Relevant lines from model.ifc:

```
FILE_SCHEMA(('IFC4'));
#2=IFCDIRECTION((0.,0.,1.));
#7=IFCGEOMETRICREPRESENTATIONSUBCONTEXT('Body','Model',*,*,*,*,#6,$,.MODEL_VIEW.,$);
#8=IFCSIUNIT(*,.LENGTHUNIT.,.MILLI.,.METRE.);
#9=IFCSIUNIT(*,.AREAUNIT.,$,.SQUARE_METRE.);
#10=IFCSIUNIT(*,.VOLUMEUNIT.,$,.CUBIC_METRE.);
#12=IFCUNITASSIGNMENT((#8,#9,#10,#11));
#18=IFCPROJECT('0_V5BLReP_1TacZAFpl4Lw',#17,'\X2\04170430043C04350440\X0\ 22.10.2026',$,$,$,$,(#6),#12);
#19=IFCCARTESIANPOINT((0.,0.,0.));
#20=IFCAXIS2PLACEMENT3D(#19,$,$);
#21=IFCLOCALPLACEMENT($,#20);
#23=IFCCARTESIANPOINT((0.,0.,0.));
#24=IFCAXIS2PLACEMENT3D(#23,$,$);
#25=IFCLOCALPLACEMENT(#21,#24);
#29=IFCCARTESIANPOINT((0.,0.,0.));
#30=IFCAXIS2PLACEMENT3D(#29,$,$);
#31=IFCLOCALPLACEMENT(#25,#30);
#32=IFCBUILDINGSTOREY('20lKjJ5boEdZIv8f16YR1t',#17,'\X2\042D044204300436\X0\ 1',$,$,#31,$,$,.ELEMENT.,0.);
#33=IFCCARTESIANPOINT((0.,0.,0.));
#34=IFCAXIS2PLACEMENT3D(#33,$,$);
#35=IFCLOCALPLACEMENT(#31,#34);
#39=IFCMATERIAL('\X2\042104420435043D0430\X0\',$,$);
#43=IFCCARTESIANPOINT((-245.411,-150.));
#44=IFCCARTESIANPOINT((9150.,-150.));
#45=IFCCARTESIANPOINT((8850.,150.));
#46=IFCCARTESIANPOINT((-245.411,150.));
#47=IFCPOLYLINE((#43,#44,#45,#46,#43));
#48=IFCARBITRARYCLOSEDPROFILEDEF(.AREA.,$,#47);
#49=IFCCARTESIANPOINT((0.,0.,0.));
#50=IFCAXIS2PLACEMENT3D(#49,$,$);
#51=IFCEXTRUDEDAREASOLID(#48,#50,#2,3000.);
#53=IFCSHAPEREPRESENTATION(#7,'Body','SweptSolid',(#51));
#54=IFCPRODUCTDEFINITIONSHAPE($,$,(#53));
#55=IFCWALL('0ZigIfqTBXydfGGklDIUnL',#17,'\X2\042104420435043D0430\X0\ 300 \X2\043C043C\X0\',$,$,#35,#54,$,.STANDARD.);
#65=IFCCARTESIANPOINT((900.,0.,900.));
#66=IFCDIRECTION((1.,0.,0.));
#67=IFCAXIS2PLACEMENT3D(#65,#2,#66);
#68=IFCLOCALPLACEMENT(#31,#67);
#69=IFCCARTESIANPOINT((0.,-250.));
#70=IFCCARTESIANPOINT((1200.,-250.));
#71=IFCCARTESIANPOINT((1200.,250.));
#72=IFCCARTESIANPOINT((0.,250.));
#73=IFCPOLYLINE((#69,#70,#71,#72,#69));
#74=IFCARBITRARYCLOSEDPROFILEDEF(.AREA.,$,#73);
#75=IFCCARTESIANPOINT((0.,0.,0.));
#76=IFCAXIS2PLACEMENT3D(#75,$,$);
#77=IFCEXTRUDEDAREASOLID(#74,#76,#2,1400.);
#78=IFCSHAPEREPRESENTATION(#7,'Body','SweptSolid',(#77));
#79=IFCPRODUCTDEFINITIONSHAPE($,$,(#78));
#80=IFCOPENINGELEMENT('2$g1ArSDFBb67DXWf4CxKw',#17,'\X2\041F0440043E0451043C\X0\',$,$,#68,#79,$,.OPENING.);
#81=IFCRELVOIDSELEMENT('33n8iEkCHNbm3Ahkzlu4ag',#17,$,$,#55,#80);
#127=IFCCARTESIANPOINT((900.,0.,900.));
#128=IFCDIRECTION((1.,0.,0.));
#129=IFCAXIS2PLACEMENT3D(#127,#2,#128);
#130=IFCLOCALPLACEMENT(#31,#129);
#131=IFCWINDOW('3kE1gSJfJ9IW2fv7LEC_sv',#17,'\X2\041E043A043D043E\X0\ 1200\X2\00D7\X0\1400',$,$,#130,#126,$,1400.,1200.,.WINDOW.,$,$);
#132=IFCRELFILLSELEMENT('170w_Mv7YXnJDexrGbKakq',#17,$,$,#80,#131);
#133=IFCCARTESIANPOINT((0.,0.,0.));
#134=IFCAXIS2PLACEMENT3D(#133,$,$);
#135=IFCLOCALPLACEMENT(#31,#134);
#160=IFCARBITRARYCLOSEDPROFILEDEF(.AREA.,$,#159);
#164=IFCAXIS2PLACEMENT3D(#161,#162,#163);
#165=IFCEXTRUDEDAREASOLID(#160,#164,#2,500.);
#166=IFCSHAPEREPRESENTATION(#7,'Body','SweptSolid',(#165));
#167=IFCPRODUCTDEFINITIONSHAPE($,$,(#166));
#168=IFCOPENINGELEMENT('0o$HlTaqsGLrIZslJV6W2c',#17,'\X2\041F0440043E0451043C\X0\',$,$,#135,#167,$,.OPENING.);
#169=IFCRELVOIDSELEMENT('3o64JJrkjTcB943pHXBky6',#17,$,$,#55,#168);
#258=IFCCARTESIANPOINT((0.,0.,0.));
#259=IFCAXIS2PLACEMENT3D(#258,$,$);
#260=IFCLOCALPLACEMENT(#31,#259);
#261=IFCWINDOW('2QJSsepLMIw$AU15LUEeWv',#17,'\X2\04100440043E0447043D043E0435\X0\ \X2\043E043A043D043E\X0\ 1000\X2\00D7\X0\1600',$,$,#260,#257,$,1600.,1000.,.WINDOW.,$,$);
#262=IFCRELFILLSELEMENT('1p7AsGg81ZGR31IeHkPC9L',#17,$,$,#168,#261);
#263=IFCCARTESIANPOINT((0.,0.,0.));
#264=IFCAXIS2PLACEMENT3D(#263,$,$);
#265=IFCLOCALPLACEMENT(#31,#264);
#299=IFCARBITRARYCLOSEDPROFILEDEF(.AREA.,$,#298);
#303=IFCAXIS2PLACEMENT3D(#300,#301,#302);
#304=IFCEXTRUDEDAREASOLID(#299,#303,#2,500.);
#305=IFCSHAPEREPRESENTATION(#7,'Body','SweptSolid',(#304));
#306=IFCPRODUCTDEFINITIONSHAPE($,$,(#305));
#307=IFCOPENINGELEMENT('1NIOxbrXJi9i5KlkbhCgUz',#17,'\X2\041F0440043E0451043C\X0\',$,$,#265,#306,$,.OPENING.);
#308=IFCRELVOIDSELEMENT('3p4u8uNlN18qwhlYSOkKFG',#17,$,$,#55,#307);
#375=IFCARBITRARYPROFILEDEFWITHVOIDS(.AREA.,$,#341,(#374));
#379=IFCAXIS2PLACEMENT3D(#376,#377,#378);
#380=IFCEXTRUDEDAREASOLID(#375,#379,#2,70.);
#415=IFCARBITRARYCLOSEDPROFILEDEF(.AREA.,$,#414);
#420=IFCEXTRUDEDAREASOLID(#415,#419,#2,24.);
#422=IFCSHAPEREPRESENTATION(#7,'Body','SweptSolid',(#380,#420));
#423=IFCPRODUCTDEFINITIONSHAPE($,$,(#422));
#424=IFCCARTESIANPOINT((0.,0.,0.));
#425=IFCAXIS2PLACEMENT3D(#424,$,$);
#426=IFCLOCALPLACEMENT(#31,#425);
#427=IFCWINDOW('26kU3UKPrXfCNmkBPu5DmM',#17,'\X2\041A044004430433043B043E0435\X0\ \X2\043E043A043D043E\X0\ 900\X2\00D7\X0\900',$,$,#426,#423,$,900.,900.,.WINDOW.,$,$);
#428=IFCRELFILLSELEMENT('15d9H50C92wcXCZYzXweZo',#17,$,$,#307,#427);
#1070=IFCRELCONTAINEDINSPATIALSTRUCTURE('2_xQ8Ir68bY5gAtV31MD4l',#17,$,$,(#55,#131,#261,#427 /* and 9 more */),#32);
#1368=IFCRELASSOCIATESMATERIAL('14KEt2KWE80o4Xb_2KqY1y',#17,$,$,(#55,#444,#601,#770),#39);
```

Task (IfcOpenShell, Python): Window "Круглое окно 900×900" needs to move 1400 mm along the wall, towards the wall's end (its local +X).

```python
import ifcopenshell
import ifcopenshell.api.geometry
import ifcopenshell.util.placement

model = ifcopenshell.open("model.ifc")

window = model.by_guid("26kU3UKPrXfCNmkBPu5DmM")
opening = window.FillsVoids[0].RelatingOpeningElement
wall = opening.VoidsElements[0].RelatingBuildingElement

wall_matrix = ifcopenshell.util.placement.get_local_placement(wall.ObjectPlacement)
shift = wall_matrix[:3, 0] * 1400.0
before = ifcopenshell.util.placement.get_local_placement(window.ObjectPlacement)[:3, 3].copy()

# The window is not placed relative to its opening, so move both.
for product in (opening, window):
    matrix = ifcopenshell.util.placement.get_local_placement(product.ObjectPlacement)
    matrix[:3, 3] += shift
    ifcopenshell.api.geometry.edit_object_placement(model, product=product, matrix=matrix, is_si=False)

after = ifcopenshell.util.placement.get_local_placement(window.ObjectPlacement)[:3, 3]
print("window moved by", (after - before).round(3) + 0.0)

model.write("model-out.ifc")
```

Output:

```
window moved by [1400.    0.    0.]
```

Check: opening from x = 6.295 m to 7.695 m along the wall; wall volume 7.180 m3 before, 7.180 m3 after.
